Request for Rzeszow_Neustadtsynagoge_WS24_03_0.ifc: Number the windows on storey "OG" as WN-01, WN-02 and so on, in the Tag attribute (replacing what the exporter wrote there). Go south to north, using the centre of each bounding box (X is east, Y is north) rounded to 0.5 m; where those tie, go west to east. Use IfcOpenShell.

First a look at what the model holds.

```python
import ifcopenshell
import ifcopenshell.util.element
import ifcopenshell.util.placement

model = ifcopenshell.open("Rzeszow_Neustadtsynagoge_WS24_03_0.ifc")
print(model.schema)
storey = next(s for s in model.by_type("IfcBuildingStorey") if s.Name == "OG")
windows = [e for e in ifcopenshell.util.element.get_decomposition(storey) if e.is_a("IfcWindow")]
for e in sorted(windows, key=lambda e: e.id()):
    origin = ifcopenshell.util.placement.get_local_placement(e.ObjectPlacement)[:3, 3]
    print(e.id(), e.Tag, e.Name, origin.round(2) + 0.0, sep=" | ")
```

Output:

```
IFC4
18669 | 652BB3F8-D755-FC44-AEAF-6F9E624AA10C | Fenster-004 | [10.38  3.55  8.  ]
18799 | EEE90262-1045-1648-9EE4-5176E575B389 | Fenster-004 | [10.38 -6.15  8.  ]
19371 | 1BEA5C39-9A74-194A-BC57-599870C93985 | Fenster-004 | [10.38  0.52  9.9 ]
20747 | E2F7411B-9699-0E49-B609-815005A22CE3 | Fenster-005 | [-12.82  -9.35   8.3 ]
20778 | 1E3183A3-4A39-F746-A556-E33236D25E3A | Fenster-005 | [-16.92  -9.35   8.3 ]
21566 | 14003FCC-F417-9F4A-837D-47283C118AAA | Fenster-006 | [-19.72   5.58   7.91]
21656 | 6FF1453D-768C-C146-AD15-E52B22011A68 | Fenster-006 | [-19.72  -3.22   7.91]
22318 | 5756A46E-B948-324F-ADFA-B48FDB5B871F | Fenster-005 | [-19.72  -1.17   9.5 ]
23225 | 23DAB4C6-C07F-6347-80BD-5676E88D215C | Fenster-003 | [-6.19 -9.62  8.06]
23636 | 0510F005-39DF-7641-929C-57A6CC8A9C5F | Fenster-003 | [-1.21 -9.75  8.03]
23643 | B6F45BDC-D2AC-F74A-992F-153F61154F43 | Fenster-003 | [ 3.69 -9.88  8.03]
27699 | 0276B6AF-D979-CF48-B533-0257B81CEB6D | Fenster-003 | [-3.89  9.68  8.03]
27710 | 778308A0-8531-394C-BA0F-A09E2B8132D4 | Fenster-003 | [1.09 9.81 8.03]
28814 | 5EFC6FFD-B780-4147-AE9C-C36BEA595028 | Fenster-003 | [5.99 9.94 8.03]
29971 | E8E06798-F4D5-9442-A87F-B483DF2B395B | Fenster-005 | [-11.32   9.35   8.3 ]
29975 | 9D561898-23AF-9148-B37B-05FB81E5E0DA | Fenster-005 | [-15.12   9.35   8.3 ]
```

```python
import ifcopenshell
import ifcopenshell.geom
import ifcopenshell.util.element
import ifcopenshell.util.shape

model = ifcopenshell.open("Rzeszow_Neustadtsynagoge_WS24_03_0.ifc")
settings = ifcopenshell.geom.settings()
settings.set("use-world-coords", True)


def centre(element):
    shape = ifcopenshell.geom.create_shape(settings, element)
    return ifcopenshell.util.shape.get_bbox_centroid(shape.geometry)


storey = next(s for s in model.by_type("IfcBuildingStorey") if s.Name == "OG")
windows = [e for e in ifcopenshell.util.element.get_decomposition(storey) if e.is_a("IfcWindow")]

# Insertion points can sit at a corner or the storey origin, so sort by the geometry (in metres).
centres = {e: centre(e) for e in windows}
windows.sort(key=lambda e: (round(centres[e][1] / 0.5), centres[e][0]))

for i, e in enumerate(windows, start=1):
    number = f"WN-{i:02d}"
    e.Tag = number
    print(e.id(), number)

model.write("Rzeszow_Neustadtsynagoge_WS24_03_0-out.ifc")
```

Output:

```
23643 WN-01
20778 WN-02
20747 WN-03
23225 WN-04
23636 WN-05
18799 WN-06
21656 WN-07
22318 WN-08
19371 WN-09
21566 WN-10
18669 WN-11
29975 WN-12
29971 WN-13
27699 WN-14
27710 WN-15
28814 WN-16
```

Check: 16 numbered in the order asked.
